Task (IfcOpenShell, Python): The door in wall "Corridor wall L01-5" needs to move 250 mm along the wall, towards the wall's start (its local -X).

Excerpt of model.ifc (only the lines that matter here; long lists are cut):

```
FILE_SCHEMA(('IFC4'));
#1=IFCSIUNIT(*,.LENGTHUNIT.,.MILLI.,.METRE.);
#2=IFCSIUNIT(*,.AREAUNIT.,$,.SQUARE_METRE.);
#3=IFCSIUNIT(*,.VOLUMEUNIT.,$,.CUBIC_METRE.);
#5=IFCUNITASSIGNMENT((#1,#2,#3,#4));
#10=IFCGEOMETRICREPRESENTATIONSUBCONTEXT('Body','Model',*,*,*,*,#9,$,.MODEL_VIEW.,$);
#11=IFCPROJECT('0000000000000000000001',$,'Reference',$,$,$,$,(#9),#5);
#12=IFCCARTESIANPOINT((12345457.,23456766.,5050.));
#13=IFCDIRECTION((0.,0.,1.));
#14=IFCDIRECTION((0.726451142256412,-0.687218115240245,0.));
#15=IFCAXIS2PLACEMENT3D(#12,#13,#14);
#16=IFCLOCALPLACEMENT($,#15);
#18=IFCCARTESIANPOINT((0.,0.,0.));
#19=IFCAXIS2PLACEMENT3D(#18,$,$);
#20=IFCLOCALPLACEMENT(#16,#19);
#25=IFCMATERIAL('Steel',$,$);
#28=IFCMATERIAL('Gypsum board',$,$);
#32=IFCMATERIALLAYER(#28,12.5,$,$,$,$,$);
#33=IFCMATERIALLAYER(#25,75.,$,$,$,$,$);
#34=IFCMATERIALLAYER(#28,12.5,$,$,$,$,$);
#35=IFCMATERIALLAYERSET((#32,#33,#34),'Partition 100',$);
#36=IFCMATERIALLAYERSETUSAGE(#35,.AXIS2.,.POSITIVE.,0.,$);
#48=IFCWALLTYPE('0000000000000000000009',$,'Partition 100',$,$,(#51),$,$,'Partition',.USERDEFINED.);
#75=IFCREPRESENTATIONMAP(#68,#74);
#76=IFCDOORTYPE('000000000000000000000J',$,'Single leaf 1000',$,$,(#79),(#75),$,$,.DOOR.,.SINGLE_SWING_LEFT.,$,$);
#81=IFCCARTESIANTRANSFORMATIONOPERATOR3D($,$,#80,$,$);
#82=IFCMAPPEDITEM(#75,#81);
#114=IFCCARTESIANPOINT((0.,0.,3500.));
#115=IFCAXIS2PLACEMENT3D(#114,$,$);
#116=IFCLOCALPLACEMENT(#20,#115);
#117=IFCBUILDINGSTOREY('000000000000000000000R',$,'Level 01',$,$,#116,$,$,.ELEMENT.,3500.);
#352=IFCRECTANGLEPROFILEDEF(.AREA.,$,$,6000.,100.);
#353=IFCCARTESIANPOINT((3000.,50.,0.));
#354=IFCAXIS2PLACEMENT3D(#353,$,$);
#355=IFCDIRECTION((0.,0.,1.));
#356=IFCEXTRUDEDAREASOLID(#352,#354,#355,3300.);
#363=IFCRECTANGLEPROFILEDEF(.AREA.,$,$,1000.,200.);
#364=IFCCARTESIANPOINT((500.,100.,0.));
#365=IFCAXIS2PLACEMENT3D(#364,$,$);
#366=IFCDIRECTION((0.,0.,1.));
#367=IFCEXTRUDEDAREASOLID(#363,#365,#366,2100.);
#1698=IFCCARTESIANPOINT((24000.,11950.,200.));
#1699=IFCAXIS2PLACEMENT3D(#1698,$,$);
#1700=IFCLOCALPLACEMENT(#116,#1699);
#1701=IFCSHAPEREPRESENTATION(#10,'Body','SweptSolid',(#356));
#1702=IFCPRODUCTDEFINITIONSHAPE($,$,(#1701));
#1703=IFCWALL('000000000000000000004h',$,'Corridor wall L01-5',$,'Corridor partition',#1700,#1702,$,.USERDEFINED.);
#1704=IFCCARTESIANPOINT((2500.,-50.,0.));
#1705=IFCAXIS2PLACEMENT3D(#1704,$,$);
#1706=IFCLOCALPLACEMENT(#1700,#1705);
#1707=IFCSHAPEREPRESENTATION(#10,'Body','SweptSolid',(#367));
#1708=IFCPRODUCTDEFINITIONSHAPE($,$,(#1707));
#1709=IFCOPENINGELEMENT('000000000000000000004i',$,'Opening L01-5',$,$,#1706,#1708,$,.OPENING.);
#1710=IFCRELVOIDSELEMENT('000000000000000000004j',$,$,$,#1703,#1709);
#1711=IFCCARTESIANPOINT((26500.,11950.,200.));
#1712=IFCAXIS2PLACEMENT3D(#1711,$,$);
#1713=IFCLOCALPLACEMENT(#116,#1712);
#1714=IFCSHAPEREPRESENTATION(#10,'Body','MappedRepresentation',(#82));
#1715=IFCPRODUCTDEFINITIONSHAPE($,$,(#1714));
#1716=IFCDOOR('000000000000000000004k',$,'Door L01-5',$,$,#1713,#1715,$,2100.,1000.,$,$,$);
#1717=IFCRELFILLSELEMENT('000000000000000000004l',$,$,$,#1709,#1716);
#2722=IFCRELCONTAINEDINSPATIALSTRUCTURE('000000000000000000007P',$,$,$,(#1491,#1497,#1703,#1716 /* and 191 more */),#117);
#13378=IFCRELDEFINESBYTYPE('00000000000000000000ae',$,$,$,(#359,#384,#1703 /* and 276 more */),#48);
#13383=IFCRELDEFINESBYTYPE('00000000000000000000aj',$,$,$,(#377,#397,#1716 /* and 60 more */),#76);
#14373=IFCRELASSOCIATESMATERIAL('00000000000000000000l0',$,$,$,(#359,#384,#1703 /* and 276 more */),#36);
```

```python
import ifcopenshell
import ifcopenshell.api.geometry
import ifcopenshell.util.placement
import ifcopenshell.util.unit

model = ifcopenshell.open("model.ifc")
unit_scale = ifcopenshell.util.unit.calculate_unit_scale(model)

door = model.by_id(1716)
opening = door.FillsVoids[0].RelatingOpeningElement
wall = opening.VoidsElements[0].RelatingBuildingElement

wall_matrix = ifcopenshell.util.placement.get_local_placement(wall.ObjectPlacement)
shift = wall_matrix[:3, 0] * -0.25 / unit_scale
before = ifcopenshell.util.placement.get_local_placement(door.ObjectPlacement)[:3, 3].copy()

# The door is not placed relative to its opening, so move both.
for product in (opening, door):
    matrix = ifcopenshell.util.placement.get_local_placement(product.ObjectPlacement)
    matrix[:3, 3] += shift
    ifcopenshell.api.geometry.edit_object_placement(model, product=product, matrix=matrix, is_si=False)

after = ifcopenshell.util.placement.get_local_placement(door.ObjectPlacement)[:3, 3]
print("door moved by", (after - before).round(3) + 0.0)

model.write("model_rev.ifc")
```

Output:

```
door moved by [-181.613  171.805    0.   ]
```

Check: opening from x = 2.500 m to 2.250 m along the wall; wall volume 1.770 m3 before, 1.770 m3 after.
